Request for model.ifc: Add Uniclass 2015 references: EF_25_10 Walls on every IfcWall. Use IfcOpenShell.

First a look at what the model holds.

```python
import ifcopenshell

model = ifcopenshell.open("model.ifc")
print(model.schema)
print("classifications:", [c.Name for c in model.by_type("IfcClassification")])
for ifc_class in ("IfcDoor", "IfcRoof", "IfcStair", "IfcWall", "IfcWindow"):
    print(ifc_class, len(model.by_type(ifc_class)))
```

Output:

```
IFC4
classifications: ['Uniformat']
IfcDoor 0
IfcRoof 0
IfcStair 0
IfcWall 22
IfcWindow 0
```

```python
import ifcopenshell
import ifcopenshell.api.classification

model = ifcopenshell.open("model.ifc")

system = ifcopenshell.api.classification.add_classification(model, classification="Uniclass 2015")

codes = {
    "IfcWall": ("EF_25_10", "Walls"),
}
for ifc_class, (code, name) in codes.items():
    products = model.by_type(ifc_class)
    ifcopenshell.api.classification.add_reference(
        model, products=products, classification=system, identification=code, name=name
    )
    print(code, len(products))

model.write("model-out.ifc")
```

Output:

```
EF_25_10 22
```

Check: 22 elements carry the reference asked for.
